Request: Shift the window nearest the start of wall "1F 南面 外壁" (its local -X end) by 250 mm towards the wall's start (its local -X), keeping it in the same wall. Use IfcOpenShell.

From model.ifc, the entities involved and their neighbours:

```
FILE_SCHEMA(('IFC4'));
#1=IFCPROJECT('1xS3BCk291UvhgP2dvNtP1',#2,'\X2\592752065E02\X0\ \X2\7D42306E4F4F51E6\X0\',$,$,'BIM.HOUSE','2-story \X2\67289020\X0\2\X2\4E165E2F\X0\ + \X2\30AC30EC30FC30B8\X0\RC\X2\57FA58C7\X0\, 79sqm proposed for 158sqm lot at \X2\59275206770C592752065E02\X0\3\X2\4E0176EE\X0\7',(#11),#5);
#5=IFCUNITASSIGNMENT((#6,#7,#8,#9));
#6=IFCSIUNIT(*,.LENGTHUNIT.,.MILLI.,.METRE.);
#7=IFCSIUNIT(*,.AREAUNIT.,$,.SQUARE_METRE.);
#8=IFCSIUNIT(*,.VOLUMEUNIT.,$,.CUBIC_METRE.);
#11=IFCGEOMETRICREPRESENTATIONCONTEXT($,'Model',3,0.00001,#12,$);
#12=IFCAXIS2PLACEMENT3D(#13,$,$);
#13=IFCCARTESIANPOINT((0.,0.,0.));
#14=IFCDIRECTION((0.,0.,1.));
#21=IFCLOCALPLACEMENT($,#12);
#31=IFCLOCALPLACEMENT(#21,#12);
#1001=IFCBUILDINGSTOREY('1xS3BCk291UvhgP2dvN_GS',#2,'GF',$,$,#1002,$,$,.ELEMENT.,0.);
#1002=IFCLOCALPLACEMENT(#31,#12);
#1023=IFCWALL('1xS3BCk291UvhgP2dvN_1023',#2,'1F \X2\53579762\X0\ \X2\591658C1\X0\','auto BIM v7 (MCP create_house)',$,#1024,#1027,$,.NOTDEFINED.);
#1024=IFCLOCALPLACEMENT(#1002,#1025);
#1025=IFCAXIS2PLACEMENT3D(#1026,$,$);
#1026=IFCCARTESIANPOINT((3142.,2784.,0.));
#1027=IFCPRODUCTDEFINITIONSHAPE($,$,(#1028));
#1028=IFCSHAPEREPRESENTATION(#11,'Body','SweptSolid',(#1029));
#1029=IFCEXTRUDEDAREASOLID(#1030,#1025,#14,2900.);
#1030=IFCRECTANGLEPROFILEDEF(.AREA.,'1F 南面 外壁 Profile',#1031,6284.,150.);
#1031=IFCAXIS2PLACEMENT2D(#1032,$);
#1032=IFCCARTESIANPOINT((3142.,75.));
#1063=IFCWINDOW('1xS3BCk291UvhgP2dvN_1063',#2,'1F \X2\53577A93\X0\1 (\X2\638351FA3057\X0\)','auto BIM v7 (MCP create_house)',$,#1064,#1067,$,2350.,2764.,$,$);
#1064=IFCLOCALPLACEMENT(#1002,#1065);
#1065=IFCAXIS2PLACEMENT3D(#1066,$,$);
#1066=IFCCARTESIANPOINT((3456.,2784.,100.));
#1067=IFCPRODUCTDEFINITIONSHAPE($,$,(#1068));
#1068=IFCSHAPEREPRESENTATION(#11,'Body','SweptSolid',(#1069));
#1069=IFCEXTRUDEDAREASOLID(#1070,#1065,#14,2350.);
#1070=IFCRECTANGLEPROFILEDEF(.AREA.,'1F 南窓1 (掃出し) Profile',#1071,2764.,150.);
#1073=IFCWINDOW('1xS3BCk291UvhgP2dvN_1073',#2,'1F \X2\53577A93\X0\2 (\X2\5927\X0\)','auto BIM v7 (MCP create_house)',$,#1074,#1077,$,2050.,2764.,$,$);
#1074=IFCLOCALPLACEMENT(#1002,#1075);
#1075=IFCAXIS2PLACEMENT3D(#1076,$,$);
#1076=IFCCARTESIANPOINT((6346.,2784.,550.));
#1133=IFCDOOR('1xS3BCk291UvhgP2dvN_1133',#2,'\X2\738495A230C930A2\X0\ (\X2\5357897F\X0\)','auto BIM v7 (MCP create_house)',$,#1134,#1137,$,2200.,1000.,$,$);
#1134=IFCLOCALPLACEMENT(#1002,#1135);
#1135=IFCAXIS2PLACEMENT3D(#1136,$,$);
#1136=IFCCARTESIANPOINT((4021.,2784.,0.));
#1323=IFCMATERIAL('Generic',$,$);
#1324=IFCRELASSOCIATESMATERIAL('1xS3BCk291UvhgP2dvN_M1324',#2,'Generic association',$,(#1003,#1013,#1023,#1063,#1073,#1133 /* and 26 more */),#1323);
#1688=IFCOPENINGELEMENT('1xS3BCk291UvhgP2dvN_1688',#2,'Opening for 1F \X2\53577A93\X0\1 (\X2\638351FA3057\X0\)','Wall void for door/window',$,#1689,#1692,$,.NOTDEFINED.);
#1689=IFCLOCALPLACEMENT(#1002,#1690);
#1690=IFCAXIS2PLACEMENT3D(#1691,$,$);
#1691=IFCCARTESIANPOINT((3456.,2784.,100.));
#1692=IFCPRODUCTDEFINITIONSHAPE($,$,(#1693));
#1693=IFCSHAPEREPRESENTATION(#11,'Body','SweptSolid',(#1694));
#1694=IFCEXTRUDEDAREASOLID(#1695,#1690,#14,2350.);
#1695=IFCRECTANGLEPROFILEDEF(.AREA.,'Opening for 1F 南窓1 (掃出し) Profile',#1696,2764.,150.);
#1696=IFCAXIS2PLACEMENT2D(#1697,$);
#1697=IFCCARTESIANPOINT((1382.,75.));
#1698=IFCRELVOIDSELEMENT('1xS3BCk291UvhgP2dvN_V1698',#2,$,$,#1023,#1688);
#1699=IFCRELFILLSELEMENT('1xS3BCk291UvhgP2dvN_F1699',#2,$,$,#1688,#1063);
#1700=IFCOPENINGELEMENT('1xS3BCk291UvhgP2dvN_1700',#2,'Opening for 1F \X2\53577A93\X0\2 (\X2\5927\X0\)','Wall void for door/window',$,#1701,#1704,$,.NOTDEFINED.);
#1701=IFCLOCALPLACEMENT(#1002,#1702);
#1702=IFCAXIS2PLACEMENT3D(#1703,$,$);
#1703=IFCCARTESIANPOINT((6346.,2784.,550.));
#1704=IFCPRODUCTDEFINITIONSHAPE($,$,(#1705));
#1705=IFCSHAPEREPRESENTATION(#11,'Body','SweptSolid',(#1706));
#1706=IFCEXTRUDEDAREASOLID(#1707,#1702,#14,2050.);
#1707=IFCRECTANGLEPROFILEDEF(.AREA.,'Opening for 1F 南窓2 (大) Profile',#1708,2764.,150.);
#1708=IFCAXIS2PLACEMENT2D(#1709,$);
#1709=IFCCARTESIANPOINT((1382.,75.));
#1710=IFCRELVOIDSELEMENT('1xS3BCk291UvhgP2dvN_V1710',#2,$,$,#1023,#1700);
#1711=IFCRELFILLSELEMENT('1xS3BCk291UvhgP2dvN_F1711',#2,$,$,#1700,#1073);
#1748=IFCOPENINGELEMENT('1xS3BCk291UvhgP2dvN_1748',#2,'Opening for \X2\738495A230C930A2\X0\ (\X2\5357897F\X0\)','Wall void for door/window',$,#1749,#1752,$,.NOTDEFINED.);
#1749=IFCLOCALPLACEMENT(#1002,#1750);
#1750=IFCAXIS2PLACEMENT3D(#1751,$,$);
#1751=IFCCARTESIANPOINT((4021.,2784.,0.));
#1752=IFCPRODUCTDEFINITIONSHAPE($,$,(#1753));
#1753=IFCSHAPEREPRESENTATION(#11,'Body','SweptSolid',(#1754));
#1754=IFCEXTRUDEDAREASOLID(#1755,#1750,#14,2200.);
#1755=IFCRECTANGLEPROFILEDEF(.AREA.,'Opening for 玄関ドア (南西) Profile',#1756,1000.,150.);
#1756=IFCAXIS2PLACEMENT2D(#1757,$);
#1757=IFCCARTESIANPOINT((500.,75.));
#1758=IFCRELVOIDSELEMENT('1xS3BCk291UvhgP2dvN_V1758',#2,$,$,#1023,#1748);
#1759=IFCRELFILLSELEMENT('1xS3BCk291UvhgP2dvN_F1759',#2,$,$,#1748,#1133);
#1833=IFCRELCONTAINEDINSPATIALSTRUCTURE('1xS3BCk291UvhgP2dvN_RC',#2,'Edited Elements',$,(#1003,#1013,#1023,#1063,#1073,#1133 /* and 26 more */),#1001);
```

```python
import ifcopenshell
import ifcopenshell.api.geometry
import ifcopenshell.util.placement
import ifcopenshell.util.unit

model = ifcopenshell.open("model.ifc")
unit_scale = ifcopenshell.util.unit.calculate_unit_scale(model)

window = model.by_guid("1xS3BCk291UvhgP2dvN_1063")
opening = window.FillsVoids[0].RelatingOpeningElement
wall = opening.VoidsElements[0].RelatingBuildingElement

wall_matrix = ifcopenshell.util.placement.get_local_placement(wall.ObjectPlacement)
shift = wall_matrix[:3, 0] * -0.25 / unit_scale
before = ifcopenshell.util.placement.get_local_placement(window.ObjectPlacement)[:3, 3].copy()

# The window is not placed relative to its opening, so move both.
for product in (opening, window):
    matrix = ifcopenshell.util.placement.get_local_placement(product.ObjectPlacement)
    matrix[:3, 3] += shift
    ifcopenshell.api.geometry.edit_object_placement(model, product=product, matrix=matrix, is_si=False)

after = ifcopenshell.util.placement.get_local_placement(window.ObjectPlacement)[:3, 3]
print("window moved by", (after - before).round(3) + 0.0)

model.write("model_rev.ifc")
```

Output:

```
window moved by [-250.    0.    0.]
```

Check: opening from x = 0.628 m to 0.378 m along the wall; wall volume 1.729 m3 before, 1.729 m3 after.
